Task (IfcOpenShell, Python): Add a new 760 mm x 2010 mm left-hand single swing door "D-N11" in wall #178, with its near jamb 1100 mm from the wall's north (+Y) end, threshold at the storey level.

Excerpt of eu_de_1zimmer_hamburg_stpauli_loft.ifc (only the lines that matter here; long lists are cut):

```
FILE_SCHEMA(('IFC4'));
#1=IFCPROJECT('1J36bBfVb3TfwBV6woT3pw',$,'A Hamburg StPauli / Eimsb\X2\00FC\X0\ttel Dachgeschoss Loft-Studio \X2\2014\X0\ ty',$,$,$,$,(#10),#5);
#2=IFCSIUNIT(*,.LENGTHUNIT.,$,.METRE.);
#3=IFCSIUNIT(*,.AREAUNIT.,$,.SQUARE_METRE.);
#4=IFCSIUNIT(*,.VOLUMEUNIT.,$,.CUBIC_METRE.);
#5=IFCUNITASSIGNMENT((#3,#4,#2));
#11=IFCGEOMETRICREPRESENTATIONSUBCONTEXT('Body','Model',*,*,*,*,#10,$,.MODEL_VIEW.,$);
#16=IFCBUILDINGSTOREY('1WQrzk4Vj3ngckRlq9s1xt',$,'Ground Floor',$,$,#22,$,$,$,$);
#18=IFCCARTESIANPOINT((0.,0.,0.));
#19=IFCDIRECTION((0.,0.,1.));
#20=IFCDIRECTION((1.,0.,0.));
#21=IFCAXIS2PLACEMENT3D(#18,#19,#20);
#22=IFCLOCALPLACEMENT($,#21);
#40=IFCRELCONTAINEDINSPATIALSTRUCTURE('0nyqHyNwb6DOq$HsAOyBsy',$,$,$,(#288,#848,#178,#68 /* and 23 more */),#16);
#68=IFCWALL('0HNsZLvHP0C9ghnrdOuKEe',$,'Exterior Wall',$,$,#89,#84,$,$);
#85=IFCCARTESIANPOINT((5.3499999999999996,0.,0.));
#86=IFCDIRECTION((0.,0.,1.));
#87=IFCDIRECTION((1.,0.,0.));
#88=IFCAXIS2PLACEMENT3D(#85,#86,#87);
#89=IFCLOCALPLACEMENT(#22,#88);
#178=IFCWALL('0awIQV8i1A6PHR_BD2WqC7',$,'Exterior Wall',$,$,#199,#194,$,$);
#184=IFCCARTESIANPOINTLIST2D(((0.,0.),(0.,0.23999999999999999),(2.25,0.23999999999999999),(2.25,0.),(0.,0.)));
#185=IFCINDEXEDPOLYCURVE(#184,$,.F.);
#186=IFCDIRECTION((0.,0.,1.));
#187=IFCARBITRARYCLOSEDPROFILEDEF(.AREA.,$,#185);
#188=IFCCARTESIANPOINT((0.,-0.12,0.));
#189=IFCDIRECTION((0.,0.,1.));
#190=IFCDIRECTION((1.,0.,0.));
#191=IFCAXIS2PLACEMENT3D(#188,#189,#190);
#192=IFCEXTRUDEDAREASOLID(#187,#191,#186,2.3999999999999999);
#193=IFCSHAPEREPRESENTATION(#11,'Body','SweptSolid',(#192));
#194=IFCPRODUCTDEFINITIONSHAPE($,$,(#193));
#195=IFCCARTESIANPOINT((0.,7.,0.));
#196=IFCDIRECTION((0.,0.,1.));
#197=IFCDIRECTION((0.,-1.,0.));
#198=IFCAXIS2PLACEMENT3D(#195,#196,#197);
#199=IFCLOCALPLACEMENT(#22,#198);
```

```python
import numpy as np
import ifcopenshell
import ifcopenshell.api.feature
import ifcopenshell.api.geometry
import ifcopenshell.api.root
import ifcopenshell.api.spatial
import ifcopenshell.geom
import ifcopenshell.util.element
import ifcopenshell.util.placement
import ifcopenshell.util.representation
import ifcopenshell.util.shape
import ifcopenshell.util.unit

model = ifcopenshell.open("eu_de_1zimmer_hamburg_stpauli_loft.ifc")
unit_scale = ifcopenshell.util.unit.calculate_unit_scale(model)
settings = ifcopenshell.geom.settings()


def volume(element):
    """Net volume in cubic metres, openings subtracted."""
    shape = ifcopenshell.geom.create_shape(settings, element)
    return ifcopenshell.util.shape.get_volume(shape.geometry)


wall = model.by_guid("0awIQV8i1A6PHR_BD2WqC7")
storey = ifcopenshell.util.element.get_container(wall, ifc_class="IfcBuildingStorey")
context = ifcopenshell.util.representation.get_context(model, "Model", "Body", "MODEL_VIEW")
before = volume(wall)

width, height, from_end, sill = 0.76, 2.01, 1.1, 0.0  # metres

# The wall runs along its own X axis, and the end named is its -X end.
wall_shape = ifcopenshell.geom.create_shape(settings, wall)
x, y, z = ifcopenshell.util.shape.get_vertices(wall_shape.geometry).T
start = x.min() + from_end
face, thickness = float(y.min()), float(y.max() - y.min())
wall_matrix = ifcopenshell.util.placement.get_local_placement(wall.ObjectPlacement)
level = ifcopenshell.util.placement.get_local_placement(storey.ObjectPlacement)[2, 3]


def in_wall(x, y):
    """Placement at x, y metres in the wall's axes, at sill height."""
    matrix = wall_matrix.copy()
    matrix[:, 3] = wall_matrix @ np.array([x / unit_scale, y / unit_scale, 0.0, 1.0])
    matrix[2, 3] = level + sill / unit_scale
    return matrix


# Opening: a box that overshoots both wall faces by 50 mm.
opening = ifcopenshell.api.root.create_entity(model, ifc_class="IfcOpeningElement", predefined_type="OPENING")
box = ifcopenshell.api.geometry.add_wall_representation(
    model, context=context, length=width, height=height, thickness=thickness + 0.1
)
ifcopenshell.api.geometry.assign_representation(model, product=opening, representation=box)
ifcopenshell.api.geometry.edit_object_placement(model, product=opening, matrix=in_wall(start, face - 0.05), is_si=False)
ifcopenshell.api.feature.add_feature(model, feature=opening, element=wall)

door = ifcopenshell.api.root.create_entity(model, ifc_class="IfcDoor", name="D-N11", predefined_type="DOOR")
door.OverallWidth, door.OverallHeight = width / unit_scale, height / unit_scale
door.OperationType = "SINGLE_SWING_LEFT"
body = ifcopenshell.api.geometry.add_door_representation(
    model,
    context=context,
    overall_width=door.OverallWidth,
    overall_height=door.OverallHeight,
    operation_type="SINGLE_SWING_LEFT",
    lining_properties={"LiningDepth": thickness / unit_scale, "ThresholdDepth": thickness / unit_scale},
)
ifcopenshell.api.geometry.assign_representation(model, product=door, representation=body)
ifcopenshell.api.spatial.assign_container(model, products=[door], relating_structure=storey)
ifcopenshell.api.feature.add_filling(model, opening=opening, element=door)

# The lining spans the wall, so the door starts at the wall face.
ifcopenshell.api.geometry.edit_object_placement(model, product=door, matrix=in_wall(start, face), is_si=False)

after = volume(wall)

print(f"wall volume {before:.3f} -> {after:.3f} m3")

model.write("eu_de_1zimmer_hamburg_stpauli_loft_updated.ifc")
```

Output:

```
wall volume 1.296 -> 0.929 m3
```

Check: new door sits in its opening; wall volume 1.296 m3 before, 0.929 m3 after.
